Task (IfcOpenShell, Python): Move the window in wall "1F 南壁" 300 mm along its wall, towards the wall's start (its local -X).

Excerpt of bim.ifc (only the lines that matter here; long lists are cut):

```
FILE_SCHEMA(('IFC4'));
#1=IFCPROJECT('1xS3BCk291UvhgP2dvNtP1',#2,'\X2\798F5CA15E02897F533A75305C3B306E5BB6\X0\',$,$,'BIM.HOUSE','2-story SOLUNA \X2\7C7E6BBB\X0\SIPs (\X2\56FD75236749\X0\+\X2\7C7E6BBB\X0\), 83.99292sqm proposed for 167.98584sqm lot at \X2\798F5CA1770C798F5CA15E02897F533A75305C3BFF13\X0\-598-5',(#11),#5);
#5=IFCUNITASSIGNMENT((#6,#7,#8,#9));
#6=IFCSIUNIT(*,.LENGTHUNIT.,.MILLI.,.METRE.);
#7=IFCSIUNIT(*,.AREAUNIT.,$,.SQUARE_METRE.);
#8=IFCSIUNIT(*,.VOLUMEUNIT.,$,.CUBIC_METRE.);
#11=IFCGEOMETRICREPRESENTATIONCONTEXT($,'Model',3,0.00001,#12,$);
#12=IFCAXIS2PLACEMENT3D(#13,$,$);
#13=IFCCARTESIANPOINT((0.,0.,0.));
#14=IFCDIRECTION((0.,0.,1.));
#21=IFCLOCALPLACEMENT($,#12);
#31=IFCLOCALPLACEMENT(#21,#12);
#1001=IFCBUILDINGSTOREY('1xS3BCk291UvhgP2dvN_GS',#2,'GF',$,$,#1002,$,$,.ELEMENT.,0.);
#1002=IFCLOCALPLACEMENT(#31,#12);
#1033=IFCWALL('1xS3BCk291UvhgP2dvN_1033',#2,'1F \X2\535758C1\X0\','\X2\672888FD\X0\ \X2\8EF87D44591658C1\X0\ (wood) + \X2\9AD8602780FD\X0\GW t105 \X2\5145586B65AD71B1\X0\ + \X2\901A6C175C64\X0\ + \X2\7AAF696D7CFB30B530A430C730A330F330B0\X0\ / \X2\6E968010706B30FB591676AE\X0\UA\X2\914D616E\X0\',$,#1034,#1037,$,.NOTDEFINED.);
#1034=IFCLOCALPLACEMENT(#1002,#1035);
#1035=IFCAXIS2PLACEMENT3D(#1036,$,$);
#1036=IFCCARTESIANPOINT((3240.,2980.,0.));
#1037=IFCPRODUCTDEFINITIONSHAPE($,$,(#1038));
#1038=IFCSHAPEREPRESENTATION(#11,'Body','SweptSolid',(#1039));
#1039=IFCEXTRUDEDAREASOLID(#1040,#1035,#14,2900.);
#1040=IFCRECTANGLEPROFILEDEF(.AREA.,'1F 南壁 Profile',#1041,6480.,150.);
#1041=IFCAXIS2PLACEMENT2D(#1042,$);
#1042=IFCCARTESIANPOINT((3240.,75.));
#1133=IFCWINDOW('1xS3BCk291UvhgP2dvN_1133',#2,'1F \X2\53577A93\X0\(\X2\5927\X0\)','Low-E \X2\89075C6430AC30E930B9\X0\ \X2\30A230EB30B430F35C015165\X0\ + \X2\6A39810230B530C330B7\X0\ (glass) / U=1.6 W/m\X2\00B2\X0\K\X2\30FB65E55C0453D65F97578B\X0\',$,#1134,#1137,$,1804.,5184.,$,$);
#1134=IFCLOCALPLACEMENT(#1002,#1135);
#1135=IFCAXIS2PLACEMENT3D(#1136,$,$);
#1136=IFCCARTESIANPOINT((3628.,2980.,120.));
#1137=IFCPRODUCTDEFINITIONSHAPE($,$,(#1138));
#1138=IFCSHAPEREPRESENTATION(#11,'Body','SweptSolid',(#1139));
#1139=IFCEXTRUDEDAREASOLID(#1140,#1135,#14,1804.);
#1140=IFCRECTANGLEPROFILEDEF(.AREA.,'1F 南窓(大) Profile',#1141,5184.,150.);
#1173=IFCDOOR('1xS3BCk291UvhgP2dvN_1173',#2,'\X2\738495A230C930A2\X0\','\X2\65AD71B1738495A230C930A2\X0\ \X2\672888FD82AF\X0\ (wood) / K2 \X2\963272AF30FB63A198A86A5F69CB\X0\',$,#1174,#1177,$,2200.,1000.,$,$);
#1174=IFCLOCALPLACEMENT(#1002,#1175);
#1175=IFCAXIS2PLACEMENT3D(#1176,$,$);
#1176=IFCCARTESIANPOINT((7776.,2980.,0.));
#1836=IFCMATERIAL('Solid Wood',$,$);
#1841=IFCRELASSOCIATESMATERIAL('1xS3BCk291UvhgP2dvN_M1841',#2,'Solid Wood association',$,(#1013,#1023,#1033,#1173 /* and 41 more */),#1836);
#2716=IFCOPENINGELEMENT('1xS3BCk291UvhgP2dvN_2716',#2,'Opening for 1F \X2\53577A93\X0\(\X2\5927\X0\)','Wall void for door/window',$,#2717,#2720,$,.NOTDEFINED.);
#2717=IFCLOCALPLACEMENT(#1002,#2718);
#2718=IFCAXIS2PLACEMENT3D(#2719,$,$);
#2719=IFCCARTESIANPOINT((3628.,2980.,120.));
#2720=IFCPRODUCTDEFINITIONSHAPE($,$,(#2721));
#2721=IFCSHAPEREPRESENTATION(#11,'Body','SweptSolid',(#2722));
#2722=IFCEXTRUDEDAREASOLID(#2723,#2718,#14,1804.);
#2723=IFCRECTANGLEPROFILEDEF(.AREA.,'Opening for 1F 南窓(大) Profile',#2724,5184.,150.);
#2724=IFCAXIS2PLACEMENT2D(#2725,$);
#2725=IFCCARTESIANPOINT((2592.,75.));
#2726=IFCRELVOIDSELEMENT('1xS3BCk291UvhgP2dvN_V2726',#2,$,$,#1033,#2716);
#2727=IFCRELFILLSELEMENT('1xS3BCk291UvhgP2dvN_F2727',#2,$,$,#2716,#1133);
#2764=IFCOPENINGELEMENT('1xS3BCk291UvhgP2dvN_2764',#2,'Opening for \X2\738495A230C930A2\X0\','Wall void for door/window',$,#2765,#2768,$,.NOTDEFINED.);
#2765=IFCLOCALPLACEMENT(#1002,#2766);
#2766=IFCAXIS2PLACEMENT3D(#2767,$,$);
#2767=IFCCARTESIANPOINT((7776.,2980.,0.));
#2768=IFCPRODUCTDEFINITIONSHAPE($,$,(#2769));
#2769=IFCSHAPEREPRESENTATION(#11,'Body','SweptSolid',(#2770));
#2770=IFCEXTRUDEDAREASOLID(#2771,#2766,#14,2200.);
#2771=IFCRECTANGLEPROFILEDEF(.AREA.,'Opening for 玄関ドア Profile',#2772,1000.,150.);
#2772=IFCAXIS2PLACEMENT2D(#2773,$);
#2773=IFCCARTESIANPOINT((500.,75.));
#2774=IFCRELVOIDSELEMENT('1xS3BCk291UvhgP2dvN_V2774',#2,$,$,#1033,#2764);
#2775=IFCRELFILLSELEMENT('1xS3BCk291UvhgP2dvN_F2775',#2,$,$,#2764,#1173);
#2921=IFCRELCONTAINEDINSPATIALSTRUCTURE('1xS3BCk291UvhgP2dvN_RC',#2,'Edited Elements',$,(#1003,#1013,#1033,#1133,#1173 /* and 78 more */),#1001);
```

```python
import ifcopenshell
import ifcopenshell.api.geometry
import ifcopenshell.util.placement

model = ifcopenshell.open("bim.ifc")

window = model.by_guid("1xS3BCk291UvhgP2dvN_1133")
opening = window.FillsVoids[0].RelatingOpeningElement
wall = opening.VoidsElements[0].RelatingBuildingElement

wall_matrix = ifcopenshell.util.placement.get_local_placement(wall.ObjectPlacement)
shift = wall_matrix[:3, 0] * -300.0
before = ifcopenshell.util.placement.get_local_placement(window.ObjectPlacement)[:3, 3].copy()

# The window is not placed relative to its opening, so move both.
for product in (opening, window):
    matrix = ifcopenshell.util.placement.get_local_placement(product.ObjectPlacement)
    matrix[:3, 3] += shift
    ifcopenshell.api.geometry.edit_object_placement(model, product=product, matrix=matrix, is_si=False)

after = ifcopenshell.util.placement.get_local_placement(window.ObjectPlacement)[:3, 3]
print("window moved by", (after - before).round(3) + 0.0)

model.write("bim-out.ifc")
```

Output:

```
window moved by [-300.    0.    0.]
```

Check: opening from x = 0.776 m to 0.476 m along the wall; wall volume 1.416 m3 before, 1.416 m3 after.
